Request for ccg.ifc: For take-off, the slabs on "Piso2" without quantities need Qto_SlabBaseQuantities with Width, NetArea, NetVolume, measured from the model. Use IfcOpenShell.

First a look at what the model holds.

```python
import ifcopenshell
import ifcopenshell.util.element
import ifcopenshell.util.unit

model = ifcopenshell.open("ccg.ifc")
print(model.schema)
for unit_type in ("LENGTHUNIT", "AREAUNIT", "VOLUMEUNIT"):
    print(unit_type, ifcopenshell.util.unit.calculate_unit_scale(model, unit_type))
storey = next(s for s in model.by_type("IfcBuildingStorey") if s.Name == "Piso2")
slabs = [e for e in ifcopenshell.util.element.get_decomposition(storey) if e.is_a("IfcSlab")]
for e in sorted(slabs, key=lambda e: e.id()):
    print(e.id(), e.is_a(), e.Name, list(ifcopenshell.util.element.get_psets(e, qtos_only=True)), sep=" | ")
```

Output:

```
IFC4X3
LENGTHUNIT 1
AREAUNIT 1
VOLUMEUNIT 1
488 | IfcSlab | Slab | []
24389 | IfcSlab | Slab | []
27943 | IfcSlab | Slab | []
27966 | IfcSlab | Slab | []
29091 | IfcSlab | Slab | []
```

```python
import ifcopenshell
import ifcopenshell.api.pset
import ifcopenshell.geom
import ifcopenshell.util.element
import ifcopenshell.util.shape
import ifcopenshell.util.unit

model = ifcopenshell.open("ccg.ifc")
unit_scale = ifcopenshell.util.unit.calculate_unit_scale(model)
area_scale = ifcopenshell.util.unit.calculate_unit_scale(model, "AREAUNIT")
volume_scale = ifcopenshell.util.unit.calculate_unit_scale(model, "VOLUMEUNIT")
settings = ifcopenshell.geom.settings()

storey = next(s for s in model.by_type("IfcBuildingStorey") if s.Name == "Piso2")
slabs = [e for e in ifcopenshell.util.element.get_decomposition(storey) if e.is_a("IfcSlab")]

for e in sorted(slabs, key=lambda e: e.id()):
    if ifcopenshell.util.element.get_psets(e, qtos_only=True, should_inherit=False):
        continue
    # Geometry comes back in metres, in the element's own axes.
    shape = ifcopenshell.geom.create_shape(settings, e)
    values = {
        "Width": ifcopenshell.util.shape.get_z(shape.geometry) / unit_scale,
        "NetArea": ifcopenshell.util.shape.get_footprint_area(shape.geometry) / area_scale,
        "NetVolume": ifcopenshell.util.shape.get_volume(shape.geometry) / volume_scale,
    }
    qto = ifcopenshell.api.pset.add_qto(model, product=e, name="Qto_SlabBaseQuantities")
    ifcopenshell.api.pset.edit_qto(model, qto=qto, properties=values)
    print(e.id(), {k: round(v, 3) for k, v in values.items()})

model.write("ccg_v2.ifc")
```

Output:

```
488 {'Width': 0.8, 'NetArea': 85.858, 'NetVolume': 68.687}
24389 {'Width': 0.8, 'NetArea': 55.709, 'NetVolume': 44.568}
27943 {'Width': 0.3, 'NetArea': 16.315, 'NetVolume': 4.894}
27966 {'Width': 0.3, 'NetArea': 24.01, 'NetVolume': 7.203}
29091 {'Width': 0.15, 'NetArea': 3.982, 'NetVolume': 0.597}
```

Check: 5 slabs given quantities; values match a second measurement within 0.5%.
